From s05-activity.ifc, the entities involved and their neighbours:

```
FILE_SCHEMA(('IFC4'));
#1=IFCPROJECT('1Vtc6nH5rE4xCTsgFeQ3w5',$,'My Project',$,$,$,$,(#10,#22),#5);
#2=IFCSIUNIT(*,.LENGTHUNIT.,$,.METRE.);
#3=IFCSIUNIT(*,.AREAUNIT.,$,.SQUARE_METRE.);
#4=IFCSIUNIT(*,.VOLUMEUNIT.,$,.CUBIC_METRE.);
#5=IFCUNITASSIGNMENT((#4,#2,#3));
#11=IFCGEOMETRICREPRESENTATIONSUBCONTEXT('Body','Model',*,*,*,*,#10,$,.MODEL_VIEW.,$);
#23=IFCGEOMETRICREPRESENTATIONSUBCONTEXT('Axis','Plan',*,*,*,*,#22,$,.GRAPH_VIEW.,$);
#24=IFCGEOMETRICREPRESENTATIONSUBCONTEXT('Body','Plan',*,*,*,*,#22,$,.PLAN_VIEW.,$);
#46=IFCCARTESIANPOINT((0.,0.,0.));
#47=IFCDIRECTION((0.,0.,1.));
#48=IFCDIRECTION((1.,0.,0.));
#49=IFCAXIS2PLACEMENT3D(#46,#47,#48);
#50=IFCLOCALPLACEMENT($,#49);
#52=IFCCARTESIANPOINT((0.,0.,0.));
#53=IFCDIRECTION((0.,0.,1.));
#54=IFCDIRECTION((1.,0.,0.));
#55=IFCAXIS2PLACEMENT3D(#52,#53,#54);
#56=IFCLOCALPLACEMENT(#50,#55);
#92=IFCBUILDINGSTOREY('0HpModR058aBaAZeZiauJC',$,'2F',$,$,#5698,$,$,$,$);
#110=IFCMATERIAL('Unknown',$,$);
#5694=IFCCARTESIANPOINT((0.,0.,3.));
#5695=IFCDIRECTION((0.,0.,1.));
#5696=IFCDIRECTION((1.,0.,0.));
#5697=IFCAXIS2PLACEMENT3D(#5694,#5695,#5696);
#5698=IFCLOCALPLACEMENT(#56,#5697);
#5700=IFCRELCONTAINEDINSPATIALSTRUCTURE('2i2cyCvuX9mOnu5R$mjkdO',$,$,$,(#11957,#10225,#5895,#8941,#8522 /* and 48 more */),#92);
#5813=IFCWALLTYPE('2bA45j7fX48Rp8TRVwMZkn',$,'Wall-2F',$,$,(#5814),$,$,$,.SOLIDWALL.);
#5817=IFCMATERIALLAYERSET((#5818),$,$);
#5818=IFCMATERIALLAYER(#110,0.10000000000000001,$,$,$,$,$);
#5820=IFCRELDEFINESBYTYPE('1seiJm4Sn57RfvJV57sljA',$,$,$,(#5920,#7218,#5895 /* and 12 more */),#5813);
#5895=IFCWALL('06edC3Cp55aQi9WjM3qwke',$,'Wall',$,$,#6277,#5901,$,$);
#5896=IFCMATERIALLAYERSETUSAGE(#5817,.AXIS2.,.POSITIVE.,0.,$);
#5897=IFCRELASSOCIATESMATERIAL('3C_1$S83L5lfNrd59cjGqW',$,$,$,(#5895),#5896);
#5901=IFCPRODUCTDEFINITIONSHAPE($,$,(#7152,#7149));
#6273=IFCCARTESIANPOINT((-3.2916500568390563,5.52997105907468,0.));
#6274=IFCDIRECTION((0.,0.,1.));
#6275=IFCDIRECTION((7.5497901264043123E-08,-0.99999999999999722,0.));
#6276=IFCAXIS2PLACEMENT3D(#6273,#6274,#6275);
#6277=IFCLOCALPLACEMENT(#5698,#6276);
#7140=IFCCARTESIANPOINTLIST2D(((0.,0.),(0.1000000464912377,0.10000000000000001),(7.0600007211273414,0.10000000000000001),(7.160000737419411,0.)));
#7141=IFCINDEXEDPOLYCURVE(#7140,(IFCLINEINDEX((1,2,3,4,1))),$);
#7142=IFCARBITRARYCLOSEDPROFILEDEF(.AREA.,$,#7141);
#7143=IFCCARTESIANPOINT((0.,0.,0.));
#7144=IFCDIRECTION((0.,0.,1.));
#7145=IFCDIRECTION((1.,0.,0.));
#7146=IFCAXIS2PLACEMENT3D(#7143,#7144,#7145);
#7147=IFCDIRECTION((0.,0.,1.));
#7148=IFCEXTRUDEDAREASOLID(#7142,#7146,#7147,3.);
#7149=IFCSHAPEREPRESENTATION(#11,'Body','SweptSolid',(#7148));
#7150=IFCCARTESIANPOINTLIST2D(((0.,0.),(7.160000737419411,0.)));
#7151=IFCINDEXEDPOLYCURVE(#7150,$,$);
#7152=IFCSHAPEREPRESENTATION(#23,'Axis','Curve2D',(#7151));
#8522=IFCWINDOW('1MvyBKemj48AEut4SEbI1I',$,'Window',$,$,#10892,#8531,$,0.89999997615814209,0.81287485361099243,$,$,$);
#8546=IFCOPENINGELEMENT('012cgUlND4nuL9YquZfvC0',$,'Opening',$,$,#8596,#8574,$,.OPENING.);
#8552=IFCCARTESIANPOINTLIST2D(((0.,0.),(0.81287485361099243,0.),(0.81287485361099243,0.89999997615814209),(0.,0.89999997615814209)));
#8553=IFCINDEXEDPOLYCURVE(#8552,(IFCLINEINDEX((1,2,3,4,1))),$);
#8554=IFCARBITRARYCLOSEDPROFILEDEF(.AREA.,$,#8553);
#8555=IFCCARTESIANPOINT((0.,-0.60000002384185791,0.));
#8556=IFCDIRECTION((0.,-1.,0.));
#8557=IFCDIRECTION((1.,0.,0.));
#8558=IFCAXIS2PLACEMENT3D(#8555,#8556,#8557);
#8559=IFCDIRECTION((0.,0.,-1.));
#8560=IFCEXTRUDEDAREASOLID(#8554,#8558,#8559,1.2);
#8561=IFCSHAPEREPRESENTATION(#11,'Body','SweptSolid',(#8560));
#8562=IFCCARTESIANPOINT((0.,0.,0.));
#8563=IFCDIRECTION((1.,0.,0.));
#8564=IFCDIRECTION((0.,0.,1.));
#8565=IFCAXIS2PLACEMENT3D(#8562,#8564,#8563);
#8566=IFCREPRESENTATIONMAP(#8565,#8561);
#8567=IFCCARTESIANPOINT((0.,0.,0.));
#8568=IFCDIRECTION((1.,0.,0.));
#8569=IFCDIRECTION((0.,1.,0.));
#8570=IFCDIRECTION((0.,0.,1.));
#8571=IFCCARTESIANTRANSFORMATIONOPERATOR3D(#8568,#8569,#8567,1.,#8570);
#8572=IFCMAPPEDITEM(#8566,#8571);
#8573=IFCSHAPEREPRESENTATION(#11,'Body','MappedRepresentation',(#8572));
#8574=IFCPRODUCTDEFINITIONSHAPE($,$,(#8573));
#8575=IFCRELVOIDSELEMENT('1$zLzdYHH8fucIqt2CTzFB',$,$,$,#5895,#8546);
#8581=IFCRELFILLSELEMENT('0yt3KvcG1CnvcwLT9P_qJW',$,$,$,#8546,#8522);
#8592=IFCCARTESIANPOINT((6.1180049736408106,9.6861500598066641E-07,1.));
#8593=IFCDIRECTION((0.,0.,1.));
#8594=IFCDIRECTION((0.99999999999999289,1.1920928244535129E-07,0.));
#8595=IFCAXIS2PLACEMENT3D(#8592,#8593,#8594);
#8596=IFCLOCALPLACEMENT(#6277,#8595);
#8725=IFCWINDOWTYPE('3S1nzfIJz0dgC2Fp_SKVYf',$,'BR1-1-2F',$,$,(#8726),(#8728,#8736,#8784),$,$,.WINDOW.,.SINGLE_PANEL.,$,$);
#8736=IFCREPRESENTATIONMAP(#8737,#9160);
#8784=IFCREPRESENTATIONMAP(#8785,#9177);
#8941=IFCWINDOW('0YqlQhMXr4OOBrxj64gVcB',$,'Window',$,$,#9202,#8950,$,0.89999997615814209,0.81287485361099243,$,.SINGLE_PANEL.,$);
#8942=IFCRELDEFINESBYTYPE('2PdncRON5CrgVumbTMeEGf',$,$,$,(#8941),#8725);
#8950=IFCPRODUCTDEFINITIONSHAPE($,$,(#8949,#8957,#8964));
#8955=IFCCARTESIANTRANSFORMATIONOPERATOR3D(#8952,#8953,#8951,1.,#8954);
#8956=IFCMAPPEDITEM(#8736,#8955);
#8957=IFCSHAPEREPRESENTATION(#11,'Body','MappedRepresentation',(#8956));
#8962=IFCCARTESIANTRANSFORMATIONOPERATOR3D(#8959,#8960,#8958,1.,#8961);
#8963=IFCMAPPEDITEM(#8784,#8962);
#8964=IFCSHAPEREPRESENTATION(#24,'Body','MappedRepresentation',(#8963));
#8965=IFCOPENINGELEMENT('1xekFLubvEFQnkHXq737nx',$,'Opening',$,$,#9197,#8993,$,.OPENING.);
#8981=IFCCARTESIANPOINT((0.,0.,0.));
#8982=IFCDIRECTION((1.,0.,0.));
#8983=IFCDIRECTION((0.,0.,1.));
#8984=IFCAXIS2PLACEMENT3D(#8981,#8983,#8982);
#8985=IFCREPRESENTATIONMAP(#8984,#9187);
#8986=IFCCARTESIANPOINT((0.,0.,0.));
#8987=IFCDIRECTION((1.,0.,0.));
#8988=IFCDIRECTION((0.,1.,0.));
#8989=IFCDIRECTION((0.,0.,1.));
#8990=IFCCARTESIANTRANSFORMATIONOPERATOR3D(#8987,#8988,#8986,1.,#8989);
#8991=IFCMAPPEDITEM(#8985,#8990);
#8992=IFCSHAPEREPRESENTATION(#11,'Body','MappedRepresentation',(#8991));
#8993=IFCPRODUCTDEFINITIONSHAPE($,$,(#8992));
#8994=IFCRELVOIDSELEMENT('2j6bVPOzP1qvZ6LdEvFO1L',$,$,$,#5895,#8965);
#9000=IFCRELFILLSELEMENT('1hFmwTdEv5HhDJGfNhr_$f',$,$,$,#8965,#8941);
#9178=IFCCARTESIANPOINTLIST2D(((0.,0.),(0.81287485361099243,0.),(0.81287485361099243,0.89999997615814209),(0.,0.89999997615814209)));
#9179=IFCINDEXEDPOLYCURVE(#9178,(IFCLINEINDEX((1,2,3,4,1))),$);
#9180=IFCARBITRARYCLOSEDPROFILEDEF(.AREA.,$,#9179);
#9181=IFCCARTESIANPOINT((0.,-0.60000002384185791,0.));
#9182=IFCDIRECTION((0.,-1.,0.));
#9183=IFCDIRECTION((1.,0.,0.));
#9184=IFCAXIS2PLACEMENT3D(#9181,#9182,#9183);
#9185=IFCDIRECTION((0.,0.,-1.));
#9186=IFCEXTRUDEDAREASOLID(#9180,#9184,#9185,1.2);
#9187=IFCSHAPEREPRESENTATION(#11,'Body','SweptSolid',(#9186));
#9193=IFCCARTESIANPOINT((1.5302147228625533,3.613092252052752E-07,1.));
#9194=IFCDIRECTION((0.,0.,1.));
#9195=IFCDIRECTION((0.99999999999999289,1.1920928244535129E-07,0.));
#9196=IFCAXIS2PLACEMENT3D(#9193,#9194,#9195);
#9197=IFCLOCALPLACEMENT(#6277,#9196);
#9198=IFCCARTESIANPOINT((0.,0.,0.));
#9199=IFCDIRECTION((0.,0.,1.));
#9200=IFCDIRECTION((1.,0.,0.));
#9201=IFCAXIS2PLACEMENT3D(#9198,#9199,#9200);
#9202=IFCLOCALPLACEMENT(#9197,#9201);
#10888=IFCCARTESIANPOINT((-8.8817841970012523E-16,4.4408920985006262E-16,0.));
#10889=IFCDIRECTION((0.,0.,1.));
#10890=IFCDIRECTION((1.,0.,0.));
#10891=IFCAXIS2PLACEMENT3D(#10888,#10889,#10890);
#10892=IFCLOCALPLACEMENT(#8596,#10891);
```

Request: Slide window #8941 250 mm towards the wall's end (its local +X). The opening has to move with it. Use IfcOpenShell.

```python
import ifcopenshell
import ifcopenshell.api.geometry
import ifcopenshell.util.placement
import ifcopenshell.util.unit

model = ifcopenshell.open("s05-activity.ifc")
unit_scale = ifcopenshell.util.unit.calculate_unit_scale(model)

window = model.by_id(8941)
opening = window.FillsVoids[0].RelatingOpeningElement
wall = opening.VoidsElements[0].RelatingBuildingElement

wall_matrix = ifcopenshell.util.placement.get_local_placement(wall.ObjectPlacement)
shift = wall_matrix[:3, 0] * 0.25 / unit_scale
before = ifcopenshell.util.placement.get_local_placement(window.ObjectPlacement)[:3, 3].copy()

# The window is placed relative to its opening, so it follows when the opening moves.
matrix = ifcopenshell.util.placement.get_local_placement(opening.ObjectPlacement)
matrix[:3, 3] += shift
ifcopenshell.api.geometry.edit_object_placement(
    model, product=opening, matrix=matrix, is_si=False, should_transform_children=True
)

after = ifcopenshell.util.placement.get_local_placement(window.ObjectPlacement)[:3, 3]
print("window moved by", (after - before).round(3) + 0.0)

model.write("s05-activity_rev.ifc")
```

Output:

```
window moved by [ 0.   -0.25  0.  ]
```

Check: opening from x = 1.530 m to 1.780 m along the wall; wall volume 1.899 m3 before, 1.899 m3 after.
